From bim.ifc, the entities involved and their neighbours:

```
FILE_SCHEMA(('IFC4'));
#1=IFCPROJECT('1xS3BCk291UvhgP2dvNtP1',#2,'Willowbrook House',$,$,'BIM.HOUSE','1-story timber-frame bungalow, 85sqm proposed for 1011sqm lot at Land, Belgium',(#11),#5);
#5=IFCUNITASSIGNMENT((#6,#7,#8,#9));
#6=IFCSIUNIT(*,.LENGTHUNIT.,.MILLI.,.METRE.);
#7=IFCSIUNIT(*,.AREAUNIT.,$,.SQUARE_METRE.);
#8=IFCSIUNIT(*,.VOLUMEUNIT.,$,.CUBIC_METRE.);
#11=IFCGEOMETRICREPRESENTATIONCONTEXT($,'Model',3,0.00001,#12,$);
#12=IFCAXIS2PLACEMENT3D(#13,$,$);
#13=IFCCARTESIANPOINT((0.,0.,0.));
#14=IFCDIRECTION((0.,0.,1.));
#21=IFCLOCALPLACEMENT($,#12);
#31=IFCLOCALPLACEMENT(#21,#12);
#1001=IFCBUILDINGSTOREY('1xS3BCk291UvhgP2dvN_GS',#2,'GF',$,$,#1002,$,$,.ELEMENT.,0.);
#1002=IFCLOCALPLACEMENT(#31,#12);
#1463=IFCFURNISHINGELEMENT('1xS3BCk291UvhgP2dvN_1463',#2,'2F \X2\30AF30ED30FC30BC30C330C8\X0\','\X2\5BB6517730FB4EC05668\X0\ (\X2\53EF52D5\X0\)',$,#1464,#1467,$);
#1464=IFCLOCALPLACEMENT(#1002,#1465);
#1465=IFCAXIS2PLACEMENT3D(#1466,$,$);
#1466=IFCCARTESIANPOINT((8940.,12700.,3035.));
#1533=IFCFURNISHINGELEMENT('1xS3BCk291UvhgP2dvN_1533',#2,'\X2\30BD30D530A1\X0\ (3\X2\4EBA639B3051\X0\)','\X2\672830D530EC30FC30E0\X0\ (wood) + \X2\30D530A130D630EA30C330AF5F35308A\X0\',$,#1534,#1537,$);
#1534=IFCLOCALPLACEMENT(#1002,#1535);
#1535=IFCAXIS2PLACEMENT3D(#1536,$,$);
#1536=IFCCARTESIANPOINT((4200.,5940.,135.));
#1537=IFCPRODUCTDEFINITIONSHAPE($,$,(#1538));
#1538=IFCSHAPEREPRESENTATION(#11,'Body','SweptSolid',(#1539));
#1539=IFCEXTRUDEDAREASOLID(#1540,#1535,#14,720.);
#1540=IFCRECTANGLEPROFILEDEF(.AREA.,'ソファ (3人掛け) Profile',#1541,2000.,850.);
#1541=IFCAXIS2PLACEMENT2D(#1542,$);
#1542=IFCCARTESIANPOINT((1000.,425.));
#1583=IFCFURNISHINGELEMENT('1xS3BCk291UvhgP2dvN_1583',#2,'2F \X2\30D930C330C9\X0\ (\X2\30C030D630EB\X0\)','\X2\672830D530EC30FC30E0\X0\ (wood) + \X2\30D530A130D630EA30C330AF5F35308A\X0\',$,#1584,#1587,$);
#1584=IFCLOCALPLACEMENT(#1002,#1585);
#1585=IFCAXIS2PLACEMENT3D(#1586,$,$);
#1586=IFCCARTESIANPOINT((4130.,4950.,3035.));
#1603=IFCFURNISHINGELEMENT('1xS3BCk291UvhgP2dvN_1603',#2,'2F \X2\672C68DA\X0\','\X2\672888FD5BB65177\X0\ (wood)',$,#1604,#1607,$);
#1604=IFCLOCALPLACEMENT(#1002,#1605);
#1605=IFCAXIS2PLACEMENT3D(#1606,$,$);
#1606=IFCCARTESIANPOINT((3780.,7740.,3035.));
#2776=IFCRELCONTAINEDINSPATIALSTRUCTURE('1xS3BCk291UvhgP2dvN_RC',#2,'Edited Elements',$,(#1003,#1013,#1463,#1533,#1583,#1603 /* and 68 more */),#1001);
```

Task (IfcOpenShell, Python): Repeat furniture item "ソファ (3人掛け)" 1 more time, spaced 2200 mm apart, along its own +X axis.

```python
import ifcopenshell
import ifcopenshell.api.geometry
import ifcopenshell.api.root
import ifcopenshell.util.element
import ifcopenshell.util.placement

model = ifcopenshell.open("bim.ifc")


def reuse_history(source, copy):
    """copy_class also copies each property set's owner history, people and application; keep the originals."""
    for rel in copy.IsDefinedBy:
        if rel.is_a("IfcRelDefinesByProperties") and (history := rel.RelatingPropertyDefinition.OwnerHistory):
            rel.RelatingPropertyDefinition.OwnerHistory = source.OwnerHistory
            ifcopenshell.util.element.remove_deep2(model, history)


source = model.by_id(1533)
base = ifcopenshell.util.placement.get_local_placement(source.ObjectPlacement)
step = base[:3, 0] * 2200.0

for i in range(1, 2):
    copy = ifcopenshell.api.root.copy_class(model, product=source)
    copy.Representation = ifcopenshell.util.element.copy_deep(
        model, source.Representation, exclude=["IfcGeometricRepresentationContext", "IfcRepresentationMap"]
    )
    reuse_history(source, copy)
    matrix = base.copy()
    matrix[:3, 3] += i * step
    print("added at", matrix[:3, 3].round(3) + 0.0)
    ifcopenshell.api.geometry.edit_object_placement(model, product=copy, matrix=matrix, is_si=False)

model.write("bim_v2.ifc")
```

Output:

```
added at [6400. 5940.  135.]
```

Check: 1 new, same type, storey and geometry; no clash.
